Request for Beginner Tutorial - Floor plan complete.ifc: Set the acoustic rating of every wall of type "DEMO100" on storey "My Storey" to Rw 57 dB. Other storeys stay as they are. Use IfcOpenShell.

First a look at what the model holds.

```python
import ifcopenshell
import ifcopenshell.util.element

model = ifcopenshell.open("Beginner Tutorial - Floor plan complete.ifc")
print(model.schema)
storey = next(s for s in model.by_type("IfcBuildingStorey") if s.Name == "My Storey")
walls = [e for e in ifcopenshell.util.element.get_decomposition(storey) if e.is_a("IfcWall")]
seen = {}
for e in walls:
    element_type = ifcopenshell.util.element.get_type(e)
    key = (element_type.Name if element_type != e and element_type else None, ifcopenshell.util.element.get_pset(e, "Pset_WallCommon", "AcousticRating"))
    seen[key] = seen.get(key, 0) + 1
for (name, value), count in sorted(seen.items(), key=str):
    print(count, "x", name, "|", value)
```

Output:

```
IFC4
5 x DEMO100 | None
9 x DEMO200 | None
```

```python
import ifcopenshell
import ifcopenshell.api.pset
import ifcopenshell.util.element

model = ifcopenshell.open("Beginner Tutorial - Floor plan complete.ifc")

storey = next(s for s in model.by_type("IfcBuildingStorey") if s.Name == "My Storey")
walls = [e for e in ifcopenshell.util.element.get_decomposition(storey) if e.is_a("IfcWall")]

count = 0
for e in walls:
    element_type = ifcopenshell.util.element.get_type(e)
    if element_type in (None, e) or element_type.Name != "DEMO100":
        continue
    # add_pset returns the element's existing set when there is one.
    pset = ifcopenshell.api.pset.add_pset(model, product=e, name="Pset_WallCommon")
    ifcopenshell.api.pset.edit_pset(model, pset=pset, properties={"AcousticRating": "Rw 57 dB"})
    count += 1

print(count, "walls updated")

model.write("Beginner Tutorial - Floor plan complete_edited.ifc")
```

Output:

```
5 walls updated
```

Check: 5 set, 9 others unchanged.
